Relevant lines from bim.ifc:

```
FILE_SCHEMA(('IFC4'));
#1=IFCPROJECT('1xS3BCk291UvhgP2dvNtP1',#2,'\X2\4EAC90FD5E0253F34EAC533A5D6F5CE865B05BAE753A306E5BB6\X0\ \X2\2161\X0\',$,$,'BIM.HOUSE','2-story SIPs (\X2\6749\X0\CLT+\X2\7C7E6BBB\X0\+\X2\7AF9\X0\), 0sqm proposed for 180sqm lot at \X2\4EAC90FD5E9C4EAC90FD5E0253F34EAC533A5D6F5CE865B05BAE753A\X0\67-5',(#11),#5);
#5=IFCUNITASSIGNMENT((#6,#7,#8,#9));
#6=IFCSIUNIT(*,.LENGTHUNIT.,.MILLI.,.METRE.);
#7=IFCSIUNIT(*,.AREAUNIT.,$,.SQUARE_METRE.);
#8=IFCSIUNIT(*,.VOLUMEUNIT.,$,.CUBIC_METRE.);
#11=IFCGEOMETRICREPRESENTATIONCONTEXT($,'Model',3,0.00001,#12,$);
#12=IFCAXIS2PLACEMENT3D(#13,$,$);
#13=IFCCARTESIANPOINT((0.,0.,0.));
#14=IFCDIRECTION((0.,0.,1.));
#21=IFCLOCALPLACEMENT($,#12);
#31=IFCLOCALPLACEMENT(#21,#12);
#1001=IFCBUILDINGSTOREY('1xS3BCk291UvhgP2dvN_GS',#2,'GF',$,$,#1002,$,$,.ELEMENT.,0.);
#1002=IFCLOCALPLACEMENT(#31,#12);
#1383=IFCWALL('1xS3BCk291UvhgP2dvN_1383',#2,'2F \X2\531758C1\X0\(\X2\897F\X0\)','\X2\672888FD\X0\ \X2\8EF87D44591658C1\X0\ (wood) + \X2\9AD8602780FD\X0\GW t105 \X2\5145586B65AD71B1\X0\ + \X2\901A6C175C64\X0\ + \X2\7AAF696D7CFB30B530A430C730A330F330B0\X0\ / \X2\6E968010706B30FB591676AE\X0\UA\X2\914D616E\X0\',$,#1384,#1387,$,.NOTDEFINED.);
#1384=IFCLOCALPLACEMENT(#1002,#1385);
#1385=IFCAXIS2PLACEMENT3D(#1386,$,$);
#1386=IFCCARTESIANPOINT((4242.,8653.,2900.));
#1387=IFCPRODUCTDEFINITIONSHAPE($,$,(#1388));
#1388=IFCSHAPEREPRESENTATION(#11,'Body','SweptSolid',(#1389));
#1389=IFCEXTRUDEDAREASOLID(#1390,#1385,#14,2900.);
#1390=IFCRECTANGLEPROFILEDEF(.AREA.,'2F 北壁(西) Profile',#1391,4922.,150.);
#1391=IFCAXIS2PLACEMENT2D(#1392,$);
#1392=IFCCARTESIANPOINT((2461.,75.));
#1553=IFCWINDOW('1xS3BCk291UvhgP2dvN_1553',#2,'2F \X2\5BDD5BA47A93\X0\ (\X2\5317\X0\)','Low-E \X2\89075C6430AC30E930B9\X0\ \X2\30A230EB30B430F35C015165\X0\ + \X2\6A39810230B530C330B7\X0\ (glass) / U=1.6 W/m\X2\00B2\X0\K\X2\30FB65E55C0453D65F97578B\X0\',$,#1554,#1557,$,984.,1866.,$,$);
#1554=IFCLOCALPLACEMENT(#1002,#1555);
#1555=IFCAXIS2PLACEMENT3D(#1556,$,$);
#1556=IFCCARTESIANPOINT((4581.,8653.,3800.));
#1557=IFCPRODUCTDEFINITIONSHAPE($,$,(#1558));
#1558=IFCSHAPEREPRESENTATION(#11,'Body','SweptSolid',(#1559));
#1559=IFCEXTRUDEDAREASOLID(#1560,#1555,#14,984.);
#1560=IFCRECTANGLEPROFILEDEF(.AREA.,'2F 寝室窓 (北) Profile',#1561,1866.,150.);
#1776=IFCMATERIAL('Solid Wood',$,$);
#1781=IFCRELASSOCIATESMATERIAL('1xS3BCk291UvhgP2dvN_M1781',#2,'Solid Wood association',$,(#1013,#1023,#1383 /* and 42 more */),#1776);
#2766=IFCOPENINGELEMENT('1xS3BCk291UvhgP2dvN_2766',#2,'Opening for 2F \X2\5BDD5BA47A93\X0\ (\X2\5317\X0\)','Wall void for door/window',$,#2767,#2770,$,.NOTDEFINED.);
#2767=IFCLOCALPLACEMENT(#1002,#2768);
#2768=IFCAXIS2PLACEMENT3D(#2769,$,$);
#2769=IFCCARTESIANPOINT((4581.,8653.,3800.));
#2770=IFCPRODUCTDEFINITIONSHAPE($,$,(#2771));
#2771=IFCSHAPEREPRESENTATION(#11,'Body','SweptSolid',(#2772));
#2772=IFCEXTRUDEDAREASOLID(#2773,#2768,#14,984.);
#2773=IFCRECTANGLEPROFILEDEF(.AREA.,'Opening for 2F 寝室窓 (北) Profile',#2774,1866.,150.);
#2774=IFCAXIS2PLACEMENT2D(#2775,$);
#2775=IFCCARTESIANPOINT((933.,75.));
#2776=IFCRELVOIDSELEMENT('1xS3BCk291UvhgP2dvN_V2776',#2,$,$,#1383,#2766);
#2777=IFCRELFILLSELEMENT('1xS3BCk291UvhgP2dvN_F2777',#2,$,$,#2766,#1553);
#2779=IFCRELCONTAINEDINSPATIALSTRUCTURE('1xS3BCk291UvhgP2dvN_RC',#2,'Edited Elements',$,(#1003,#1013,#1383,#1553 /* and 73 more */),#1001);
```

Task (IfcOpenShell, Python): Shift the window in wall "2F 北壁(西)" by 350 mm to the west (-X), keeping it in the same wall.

```python
import ifcopenshell
import ifcopenshell.api.geometry
import ifcopenshell.util.placement

model = ifcopenshell.open("bim.ifc")

window = model.by_guid("1xS3BCk291UvhgP2dvN_1553")
opening = window.FillsVoids[0].RelatingOpeningElement
wall = opening.VoidsElements[0].RelatingBuildingElement

wall_matrix = ifcopenshell.util.placement.get_local_placement(wall.ObjectPlacement)
shift = wall_matrix[:3, 0] * -350.0
before = ifcopenshell.util.placement.get_local_placement(window.ObjectPlacement)[:3, 3].copy()

# The window is not placed relative to its opening, so move both.
for product in (opening, window):
    matrix = ifcopenshell.util.placement.get_local_placement(product.ObjectPlacement)
    matrix[:3, 3] += shift
    ifcopenshell.api.geometry.edit_object_placement(model, product=product, matrix=matrix, is_si=False)

after = ifcopenshell.util.placement.get_local_placement(window.ObjectPlacement)[:3, 3]
print("window moved by", (after - before).round(3) + 0.0)

model.write("bim-out.ifc")
```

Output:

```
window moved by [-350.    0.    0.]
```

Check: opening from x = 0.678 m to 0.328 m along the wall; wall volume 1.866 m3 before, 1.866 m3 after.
